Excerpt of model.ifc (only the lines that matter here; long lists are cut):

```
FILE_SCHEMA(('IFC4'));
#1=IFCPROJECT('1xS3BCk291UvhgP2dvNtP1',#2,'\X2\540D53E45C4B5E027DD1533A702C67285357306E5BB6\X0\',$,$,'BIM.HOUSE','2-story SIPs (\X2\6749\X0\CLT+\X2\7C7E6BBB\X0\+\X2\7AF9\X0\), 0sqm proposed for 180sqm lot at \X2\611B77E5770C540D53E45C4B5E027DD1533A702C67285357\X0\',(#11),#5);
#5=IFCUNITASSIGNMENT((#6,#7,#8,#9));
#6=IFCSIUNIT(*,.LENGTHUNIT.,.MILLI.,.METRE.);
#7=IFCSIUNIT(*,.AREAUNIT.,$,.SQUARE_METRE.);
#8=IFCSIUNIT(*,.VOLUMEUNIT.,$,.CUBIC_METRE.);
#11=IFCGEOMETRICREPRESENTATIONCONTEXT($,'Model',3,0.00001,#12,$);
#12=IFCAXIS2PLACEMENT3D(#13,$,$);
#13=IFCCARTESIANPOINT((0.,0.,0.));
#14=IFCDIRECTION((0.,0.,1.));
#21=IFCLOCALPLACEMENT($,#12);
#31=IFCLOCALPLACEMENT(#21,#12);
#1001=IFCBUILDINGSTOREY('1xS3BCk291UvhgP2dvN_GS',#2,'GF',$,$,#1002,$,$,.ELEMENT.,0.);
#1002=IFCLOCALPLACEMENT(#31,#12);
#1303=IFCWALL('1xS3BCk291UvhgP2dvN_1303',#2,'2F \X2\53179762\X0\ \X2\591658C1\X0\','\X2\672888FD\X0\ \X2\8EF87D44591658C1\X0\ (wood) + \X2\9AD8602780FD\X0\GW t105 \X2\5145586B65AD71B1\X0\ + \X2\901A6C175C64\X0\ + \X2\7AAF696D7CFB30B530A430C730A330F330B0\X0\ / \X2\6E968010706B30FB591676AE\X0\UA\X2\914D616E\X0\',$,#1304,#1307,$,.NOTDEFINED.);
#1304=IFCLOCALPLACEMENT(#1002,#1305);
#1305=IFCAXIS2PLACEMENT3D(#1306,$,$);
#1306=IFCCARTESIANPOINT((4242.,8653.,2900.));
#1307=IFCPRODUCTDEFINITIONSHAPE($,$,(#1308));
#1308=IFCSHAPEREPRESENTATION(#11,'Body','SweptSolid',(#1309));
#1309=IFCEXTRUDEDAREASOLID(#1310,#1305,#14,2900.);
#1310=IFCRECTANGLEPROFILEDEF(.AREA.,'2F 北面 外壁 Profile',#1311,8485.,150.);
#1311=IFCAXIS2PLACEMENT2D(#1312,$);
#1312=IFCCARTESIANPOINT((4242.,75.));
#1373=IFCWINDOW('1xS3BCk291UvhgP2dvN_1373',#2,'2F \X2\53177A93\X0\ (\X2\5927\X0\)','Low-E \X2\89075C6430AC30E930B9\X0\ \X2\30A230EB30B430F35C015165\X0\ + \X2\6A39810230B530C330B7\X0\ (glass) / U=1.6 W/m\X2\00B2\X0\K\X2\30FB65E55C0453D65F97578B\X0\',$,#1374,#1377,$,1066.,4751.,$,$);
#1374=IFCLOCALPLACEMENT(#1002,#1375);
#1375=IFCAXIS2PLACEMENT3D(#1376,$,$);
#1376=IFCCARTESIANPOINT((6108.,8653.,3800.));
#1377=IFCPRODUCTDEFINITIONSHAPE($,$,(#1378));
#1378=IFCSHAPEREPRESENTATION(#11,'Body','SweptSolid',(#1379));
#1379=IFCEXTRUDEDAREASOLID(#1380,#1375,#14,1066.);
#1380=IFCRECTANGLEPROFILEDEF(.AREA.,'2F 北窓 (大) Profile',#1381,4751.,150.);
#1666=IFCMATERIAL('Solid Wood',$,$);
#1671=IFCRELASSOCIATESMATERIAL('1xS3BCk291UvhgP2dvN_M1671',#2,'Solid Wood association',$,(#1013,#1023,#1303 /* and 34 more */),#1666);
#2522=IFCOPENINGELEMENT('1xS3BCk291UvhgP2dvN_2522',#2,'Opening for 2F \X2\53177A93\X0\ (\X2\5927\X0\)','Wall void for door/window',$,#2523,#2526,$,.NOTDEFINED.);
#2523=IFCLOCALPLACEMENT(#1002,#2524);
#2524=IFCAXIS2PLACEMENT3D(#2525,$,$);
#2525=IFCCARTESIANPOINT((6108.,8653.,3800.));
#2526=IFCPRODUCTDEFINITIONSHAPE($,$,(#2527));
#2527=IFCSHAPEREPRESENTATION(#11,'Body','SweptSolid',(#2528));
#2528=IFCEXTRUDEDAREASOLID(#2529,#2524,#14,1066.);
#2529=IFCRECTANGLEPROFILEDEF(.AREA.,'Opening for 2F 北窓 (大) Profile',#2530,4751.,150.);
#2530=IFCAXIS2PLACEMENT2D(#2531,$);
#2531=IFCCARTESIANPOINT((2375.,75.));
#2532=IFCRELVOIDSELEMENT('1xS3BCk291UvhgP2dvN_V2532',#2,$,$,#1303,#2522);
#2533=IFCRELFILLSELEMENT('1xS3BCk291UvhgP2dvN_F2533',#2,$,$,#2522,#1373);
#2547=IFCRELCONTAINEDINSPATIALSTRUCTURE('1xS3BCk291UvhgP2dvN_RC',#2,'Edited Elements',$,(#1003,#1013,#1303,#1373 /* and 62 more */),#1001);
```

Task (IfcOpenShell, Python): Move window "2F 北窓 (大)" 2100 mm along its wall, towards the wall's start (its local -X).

```python
import ifcopenshell
import ifcopenshell.api.geometry
import ifcopenshell.util.placement
import ifcopenshell.util.unit

model = ifcopenshell.open("model.ifc")
unit_scale = ifcopenshell.util.unit.calculate_unit_scale(model)

window = model.by_guid("1xS3BCk291UvhgP2dvN_1373")
opening = window.FillsVoids[0].RelatingOpeningElement
wall = opening.VoidsElements[0].RelatingBuildingElement

wall_matrix = ifcopenshell.util.placement.get_local_placement(wall.ObjectPlacement)
shift = wall_matrix[:3, 0] * -2.1 / unit_scale
before = ifcopenshell.util.placement.get_local_placement(window.ObjectPlacement)[:3, 3].copy()

# The window is not placed relative to its opening, so move both.
for product in (opening, window):
    matrix = ifcopenshell.util.placement.get_local_placement(product.ObjectPlacement)
    matrix[:3, 3] += shift
    ifcopenshell.api.geometry.edit_object_placement(model, product=product, matrix=matrix, is_si=False)

after = ifcopenshell.util.placement.get_local_placement(window.ObjectPlacement)[:3, 3]
print("window moved by", (after - before).round(3) + 0.0)

model.write("model_updated.ifc")
```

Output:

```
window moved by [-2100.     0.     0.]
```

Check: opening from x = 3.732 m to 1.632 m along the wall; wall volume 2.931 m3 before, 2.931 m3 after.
